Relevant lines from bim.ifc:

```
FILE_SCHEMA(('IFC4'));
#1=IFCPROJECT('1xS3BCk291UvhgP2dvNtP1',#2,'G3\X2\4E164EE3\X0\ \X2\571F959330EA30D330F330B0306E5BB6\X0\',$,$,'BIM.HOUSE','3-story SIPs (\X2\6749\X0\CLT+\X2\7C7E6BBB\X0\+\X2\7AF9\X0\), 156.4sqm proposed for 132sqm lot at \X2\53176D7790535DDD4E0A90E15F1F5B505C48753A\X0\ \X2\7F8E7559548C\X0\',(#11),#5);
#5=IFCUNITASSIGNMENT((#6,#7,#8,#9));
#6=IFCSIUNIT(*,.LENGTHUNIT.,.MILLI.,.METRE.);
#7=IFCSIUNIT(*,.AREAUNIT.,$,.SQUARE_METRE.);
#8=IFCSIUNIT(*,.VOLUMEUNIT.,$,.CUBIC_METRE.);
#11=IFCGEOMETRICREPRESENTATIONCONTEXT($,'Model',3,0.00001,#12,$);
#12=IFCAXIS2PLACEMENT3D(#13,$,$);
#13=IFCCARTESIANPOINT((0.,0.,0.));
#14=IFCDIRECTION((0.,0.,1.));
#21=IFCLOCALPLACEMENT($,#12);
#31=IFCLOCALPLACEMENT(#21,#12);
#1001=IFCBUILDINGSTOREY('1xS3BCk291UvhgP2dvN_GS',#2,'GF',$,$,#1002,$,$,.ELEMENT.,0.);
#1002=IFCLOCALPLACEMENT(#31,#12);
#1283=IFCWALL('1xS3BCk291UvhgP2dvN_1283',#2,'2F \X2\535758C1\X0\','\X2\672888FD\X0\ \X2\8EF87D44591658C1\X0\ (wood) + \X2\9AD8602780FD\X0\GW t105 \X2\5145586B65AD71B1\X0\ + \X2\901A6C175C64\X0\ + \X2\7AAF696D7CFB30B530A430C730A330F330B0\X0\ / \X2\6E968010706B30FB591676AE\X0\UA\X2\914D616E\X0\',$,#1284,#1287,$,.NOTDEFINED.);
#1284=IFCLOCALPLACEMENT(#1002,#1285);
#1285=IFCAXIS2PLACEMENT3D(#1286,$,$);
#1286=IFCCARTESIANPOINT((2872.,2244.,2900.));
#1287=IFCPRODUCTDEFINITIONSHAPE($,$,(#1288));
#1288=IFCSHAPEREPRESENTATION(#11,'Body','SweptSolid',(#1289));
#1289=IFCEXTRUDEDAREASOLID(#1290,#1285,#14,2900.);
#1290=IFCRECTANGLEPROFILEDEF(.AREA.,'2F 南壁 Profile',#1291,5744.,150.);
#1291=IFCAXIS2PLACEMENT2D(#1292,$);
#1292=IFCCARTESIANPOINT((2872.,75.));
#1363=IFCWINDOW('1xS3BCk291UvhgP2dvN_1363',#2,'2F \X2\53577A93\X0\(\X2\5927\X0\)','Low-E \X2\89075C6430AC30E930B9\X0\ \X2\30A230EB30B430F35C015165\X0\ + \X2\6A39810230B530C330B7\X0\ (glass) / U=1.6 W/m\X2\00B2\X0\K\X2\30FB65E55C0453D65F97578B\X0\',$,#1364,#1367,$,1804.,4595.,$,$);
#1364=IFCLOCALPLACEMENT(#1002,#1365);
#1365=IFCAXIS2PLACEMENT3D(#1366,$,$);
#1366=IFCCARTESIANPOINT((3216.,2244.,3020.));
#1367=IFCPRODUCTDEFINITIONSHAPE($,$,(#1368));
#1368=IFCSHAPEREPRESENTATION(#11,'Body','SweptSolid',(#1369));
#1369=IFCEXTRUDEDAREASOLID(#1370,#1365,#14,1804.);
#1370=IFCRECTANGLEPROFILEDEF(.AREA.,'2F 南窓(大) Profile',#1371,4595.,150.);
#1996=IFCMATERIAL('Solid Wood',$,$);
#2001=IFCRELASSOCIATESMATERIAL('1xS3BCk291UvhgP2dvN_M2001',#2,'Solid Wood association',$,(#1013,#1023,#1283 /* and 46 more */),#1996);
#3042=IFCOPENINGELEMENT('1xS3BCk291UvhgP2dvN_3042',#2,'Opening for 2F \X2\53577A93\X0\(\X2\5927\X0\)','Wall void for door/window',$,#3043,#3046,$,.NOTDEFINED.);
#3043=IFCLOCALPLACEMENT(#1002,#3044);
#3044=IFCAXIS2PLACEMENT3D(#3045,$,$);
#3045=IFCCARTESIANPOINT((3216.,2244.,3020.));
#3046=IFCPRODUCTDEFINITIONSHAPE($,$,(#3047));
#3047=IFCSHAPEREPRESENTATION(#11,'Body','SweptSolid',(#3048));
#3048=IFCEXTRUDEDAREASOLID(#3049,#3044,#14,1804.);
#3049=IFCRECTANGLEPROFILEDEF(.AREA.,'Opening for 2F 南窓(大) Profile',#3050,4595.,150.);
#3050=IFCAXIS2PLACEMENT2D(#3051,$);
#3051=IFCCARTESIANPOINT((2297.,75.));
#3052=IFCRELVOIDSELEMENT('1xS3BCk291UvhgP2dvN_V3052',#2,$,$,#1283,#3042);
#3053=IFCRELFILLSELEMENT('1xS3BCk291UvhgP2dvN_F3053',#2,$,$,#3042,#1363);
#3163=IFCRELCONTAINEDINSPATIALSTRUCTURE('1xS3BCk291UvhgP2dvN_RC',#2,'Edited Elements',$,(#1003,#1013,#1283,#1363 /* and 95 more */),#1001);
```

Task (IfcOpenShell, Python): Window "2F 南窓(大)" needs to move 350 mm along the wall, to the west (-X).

```python
import ifcopenshell
import ifcopenshell.api.geometry
import ifcopenshell.util.placement
import ifcopenshell.util.unit

model = ifcopenshell.open("bim.ifc")
unit_scale = ifcopenshell.util.unit.calculate_unit_scale(model)

window = model.by_id(1363)
opening = window.FillsVoids[0].RelatingOpeningElement
wall = opening.VoidsElements[0].RelatingBuildingElement

wall_matrix = ifcopenshell.util.placement.get_local_placement(wall.ObjectPlacement)
shift = wall_matrix[:3, 0] * -0.35 / unit_scale
before = ifcopenshell.util.placement.get_local_placement(window.ObjectPlacement)[:3, 3].copy()

# The window is not placed relative to its opening, so move both.
for product in (opening, window):
    matrix = ifcopenshell.util.placement.get_local_placement(product.ObjectPlacement)
    matrix[:3, 3] += shift
    ifcopenshell.api.geometry.edit_object_placement(model, product=product, matrix=matrix, is_si=False)

after = ifcopenshell.util.placement.get_local_placement(window.ObjectPlacement)[:3, 3]
print("window moved by", (after - before).round(3) + 0.0)

model.write("bim_updated.ifc")
```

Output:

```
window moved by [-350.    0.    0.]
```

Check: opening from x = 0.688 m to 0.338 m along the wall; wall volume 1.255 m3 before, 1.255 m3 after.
